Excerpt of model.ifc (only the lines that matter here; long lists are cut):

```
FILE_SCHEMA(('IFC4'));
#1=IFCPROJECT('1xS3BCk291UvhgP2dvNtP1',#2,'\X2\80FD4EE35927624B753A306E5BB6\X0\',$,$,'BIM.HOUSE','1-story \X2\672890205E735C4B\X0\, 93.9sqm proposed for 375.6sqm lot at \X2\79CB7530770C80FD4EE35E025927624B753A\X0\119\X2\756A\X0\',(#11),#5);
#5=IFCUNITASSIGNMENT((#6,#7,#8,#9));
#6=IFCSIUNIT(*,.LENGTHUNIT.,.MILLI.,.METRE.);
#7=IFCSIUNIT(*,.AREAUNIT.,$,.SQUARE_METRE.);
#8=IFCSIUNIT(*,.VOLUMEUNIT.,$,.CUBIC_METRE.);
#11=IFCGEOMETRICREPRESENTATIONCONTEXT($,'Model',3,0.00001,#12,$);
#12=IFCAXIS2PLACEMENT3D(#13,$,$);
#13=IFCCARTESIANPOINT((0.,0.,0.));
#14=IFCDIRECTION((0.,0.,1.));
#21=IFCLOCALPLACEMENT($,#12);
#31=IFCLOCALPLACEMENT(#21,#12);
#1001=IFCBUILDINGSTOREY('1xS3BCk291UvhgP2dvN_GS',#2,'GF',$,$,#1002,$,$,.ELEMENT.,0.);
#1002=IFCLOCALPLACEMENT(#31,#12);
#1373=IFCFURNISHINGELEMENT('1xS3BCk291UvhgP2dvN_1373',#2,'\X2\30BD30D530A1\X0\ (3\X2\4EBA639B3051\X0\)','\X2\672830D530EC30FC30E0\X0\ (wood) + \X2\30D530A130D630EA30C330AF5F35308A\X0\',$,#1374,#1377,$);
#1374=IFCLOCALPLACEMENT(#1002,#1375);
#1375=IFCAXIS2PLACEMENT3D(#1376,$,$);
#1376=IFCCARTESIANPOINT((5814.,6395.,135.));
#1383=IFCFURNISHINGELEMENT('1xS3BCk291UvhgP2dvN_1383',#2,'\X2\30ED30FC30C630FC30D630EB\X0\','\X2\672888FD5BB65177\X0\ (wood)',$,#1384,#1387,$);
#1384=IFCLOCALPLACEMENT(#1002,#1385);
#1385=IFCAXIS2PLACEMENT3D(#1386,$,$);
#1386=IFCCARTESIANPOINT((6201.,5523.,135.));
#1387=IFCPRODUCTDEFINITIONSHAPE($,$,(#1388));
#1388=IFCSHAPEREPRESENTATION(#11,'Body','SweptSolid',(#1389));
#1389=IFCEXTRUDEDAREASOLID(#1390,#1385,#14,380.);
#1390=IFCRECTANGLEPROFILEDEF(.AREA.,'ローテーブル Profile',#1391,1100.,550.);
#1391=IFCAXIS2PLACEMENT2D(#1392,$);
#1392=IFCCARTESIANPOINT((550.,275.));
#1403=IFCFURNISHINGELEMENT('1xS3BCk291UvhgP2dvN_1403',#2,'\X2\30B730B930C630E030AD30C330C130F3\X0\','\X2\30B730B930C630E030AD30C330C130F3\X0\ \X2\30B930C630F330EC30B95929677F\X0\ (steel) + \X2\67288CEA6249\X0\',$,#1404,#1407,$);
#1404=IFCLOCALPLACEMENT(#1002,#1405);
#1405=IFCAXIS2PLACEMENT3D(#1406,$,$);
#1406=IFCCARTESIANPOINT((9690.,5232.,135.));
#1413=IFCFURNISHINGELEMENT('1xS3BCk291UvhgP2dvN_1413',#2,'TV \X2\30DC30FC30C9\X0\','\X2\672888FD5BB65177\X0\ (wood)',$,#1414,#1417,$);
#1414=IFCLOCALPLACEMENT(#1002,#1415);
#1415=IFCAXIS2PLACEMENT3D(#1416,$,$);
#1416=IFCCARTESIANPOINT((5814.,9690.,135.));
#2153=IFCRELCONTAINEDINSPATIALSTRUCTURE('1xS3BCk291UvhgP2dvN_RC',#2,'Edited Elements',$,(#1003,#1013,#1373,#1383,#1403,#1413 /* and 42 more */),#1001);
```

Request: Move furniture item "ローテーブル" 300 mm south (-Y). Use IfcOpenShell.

```python
import ifcopenshell
import ifcopenshell.api.geometry
import ifcopenshell.util.placement

model = ifcopenshell.open("model.ifc")

item = model.by_id(1383)
matrix = ifcopenshell.util.placement.get_local_placement(item.ObjectPlacement)
matrix[1, 3] -= 300.0
ifcopenshell.api.geometry.edit_object_placement(model, product=item, matrix=matrix, is_si=False)

print(ifcopenshell.util.placement.get_local_placement(item.ObjectPlacement).round(3) + 0.0)

model.write("model_v2.ifc")
```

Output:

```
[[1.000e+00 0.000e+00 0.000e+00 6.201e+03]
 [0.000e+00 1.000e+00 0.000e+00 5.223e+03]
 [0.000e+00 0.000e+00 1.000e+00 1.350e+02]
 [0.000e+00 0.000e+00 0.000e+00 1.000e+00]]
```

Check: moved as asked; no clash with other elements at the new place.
